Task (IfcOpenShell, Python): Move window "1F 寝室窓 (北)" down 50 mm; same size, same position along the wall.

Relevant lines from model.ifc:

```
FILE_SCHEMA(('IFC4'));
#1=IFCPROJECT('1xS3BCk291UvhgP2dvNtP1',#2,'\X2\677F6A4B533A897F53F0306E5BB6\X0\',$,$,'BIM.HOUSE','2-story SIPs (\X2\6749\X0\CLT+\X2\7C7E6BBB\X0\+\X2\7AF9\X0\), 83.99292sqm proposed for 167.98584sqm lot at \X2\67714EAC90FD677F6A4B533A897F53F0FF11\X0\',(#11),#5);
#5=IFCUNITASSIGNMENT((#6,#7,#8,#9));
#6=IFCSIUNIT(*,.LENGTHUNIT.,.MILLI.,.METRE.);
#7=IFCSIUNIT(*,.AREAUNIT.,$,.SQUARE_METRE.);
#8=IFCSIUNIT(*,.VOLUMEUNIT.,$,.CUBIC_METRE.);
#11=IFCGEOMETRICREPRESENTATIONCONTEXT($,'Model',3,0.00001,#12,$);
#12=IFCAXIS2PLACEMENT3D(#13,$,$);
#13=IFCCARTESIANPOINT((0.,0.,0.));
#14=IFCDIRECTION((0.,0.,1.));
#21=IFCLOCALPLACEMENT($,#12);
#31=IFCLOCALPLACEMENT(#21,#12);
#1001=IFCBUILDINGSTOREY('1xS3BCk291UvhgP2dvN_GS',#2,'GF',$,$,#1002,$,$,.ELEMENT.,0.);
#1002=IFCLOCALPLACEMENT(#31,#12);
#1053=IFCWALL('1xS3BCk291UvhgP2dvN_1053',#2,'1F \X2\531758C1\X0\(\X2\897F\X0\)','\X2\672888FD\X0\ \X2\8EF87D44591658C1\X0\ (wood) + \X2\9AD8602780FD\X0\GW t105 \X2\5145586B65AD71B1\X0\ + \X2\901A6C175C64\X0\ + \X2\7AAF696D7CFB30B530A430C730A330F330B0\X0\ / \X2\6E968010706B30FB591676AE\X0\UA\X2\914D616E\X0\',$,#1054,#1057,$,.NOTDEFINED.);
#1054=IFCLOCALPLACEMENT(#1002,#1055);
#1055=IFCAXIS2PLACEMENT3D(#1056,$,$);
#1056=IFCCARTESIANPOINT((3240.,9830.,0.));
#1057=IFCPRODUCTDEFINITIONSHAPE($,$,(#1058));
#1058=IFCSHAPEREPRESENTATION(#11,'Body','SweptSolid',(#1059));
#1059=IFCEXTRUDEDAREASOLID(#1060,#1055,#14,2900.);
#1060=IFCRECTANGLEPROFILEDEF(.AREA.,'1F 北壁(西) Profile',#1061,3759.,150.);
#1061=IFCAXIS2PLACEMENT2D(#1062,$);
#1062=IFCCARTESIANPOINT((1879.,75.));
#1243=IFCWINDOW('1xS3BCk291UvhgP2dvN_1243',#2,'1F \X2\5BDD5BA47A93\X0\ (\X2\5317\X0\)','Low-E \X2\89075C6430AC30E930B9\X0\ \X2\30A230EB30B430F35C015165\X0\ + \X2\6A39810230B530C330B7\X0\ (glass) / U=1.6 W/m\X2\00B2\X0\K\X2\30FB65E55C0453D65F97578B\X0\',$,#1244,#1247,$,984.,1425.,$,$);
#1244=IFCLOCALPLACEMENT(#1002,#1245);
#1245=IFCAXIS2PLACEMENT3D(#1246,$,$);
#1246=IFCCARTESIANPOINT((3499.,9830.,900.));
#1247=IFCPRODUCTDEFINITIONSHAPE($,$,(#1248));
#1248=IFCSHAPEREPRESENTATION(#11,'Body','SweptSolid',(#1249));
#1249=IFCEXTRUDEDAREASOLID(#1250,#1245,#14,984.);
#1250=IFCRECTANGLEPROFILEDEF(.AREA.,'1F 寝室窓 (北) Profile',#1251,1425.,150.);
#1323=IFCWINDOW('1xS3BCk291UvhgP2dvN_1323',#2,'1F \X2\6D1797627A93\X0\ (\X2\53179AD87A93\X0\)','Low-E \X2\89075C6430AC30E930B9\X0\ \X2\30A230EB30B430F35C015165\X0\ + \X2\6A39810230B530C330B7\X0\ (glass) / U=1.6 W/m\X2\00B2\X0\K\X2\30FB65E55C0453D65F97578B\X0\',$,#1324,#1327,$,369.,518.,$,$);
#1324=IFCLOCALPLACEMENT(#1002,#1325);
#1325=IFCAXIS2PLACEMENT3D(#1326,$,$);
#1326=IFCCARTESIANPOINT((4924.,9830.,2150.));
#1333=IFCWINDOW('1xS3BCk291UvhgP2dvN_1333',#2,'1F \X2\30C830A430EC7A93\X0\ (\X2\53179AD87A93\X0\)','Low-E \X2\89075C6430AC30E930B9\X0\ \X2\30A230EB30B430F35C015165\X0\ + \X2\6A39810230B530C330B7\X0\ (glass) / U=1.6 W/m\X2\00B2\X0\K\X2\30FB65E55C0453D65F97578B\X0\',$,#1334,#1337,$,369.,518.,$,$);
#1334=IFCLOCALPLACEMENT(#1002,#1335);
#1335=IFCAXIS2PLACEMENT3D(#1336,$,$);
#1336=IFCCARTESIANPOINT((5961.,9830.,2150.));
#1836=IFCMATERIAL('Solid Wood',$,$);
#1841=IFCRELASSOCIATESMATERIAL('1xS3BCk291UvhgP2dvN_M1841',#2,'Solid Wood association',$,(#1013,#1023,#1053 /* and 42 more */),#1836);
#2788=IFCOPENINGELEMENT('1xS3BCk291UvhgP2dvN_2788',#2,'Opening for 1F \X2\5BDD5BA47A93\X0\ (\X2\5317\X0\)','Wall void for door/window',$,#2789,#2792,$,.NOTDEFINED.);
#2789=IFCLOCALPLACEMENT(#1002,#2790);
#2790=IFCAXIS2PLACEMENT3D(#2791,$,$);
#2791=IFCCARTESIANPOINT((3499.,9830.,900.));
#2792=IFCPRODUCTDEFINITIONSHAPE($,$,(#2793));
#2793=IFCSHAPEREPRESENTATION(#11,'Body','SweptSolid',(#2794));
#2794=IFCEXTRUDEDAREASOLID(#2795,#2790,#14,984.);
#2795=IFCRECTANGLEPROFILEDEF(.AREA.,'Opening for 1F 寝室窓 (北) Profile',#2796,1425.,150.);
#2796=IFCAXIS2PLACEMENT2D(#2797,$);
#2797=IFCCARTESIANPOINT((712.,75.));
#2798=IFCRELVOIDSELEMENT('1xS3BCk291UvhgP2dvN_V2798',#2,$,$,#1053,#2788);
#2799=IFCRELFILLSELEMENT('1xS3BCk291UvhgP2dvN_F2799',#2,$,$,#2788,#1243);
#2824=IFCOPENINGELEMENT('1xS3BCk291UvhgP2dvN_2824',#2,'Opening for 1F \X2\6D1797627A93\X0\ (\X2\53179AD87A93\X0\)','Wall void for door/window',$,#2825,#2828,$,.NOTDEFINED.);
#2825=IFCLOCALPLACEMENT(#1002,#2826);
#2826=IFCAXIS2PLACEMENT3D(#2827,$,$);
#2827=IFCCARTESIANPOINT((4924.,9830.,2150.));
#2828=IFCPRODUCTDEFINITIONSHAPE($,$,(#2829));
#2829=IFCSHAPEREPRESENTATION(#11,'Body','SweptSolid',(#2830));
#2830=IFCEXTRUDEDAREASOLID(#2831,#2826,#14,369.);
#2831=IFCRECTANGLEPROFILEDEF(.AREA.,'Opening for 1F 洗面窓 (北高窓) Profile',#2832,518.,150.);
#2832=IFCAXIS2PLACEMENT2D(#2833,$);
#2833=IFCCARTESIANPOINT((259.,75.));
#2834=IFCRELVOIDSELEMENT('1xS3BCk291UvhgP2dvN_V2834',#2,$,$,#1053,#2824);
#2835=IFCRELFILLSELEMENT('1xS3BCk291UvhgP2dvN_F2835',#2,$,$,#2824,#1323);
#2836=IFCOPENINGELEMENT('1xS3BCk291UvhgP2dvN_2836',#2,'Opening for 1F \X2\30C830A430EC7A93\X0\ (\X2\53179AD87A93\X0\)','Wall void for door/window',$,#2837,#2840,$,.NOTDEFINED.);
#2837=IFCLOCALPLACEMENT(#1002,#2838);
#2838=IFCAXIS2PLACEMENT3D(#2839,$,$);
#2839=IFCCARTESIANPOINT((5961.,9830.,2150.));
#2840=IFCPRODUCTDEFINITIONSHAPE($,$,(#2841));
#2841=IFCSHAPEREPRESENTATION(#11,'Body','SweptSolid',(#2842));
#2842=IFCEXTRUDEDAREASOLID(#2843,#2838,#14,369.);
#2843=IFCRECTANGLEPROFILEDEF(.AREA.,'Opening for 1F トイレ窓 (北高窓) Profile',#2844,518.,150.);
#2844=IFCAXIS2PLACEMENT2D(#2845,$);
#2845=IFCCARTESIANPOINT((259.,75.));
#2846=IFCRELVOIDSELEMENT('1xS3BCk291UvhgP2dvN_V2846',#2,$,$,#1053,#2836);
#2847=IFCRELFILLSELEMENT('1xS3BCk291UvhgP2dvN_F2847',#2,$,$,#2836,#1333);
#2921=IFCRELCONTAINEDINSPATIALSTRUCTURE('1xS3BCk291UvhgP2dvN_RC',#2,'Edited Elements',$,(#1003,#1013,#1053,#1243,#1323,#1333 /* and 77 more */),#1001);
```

```python
import numpy as np
import ifcopenshell
import ifcopenshell.api.geometry
import ifcopenshell.util.placement
import ifcopenshell.util.unit

model = ifcopenshell.open("model.ifc")
unit_scale = ifcopenshell.util.unit.calculate_unit_scale(model)

window = model.by_guid("1xS3BCk291UvhgP2dvN_1243")
opening = window.FillsVoids[0].RelatingOpeningElement
dz = -0.05 / unit_scale

shift = np.array([0.0, 0.0, dz])
# The window is not placed relative to its opening, so move both.
for product in (opening, window):
    matrix = ifcopenshell.util.placement.get_local_placement(product.ObjectPlacement)
    matrix[:3, 3] += shift
    ifcopenshell.api.geometry.edit_object_placement(model, product=product, matrix=matrix, is_si=False)

print(f"moved by {dz * unit_scale:+.3f} m")

model.write("model-out.ifc")
```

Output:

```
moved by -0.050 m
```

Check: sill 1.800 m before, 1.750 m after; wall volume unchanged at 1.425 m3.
